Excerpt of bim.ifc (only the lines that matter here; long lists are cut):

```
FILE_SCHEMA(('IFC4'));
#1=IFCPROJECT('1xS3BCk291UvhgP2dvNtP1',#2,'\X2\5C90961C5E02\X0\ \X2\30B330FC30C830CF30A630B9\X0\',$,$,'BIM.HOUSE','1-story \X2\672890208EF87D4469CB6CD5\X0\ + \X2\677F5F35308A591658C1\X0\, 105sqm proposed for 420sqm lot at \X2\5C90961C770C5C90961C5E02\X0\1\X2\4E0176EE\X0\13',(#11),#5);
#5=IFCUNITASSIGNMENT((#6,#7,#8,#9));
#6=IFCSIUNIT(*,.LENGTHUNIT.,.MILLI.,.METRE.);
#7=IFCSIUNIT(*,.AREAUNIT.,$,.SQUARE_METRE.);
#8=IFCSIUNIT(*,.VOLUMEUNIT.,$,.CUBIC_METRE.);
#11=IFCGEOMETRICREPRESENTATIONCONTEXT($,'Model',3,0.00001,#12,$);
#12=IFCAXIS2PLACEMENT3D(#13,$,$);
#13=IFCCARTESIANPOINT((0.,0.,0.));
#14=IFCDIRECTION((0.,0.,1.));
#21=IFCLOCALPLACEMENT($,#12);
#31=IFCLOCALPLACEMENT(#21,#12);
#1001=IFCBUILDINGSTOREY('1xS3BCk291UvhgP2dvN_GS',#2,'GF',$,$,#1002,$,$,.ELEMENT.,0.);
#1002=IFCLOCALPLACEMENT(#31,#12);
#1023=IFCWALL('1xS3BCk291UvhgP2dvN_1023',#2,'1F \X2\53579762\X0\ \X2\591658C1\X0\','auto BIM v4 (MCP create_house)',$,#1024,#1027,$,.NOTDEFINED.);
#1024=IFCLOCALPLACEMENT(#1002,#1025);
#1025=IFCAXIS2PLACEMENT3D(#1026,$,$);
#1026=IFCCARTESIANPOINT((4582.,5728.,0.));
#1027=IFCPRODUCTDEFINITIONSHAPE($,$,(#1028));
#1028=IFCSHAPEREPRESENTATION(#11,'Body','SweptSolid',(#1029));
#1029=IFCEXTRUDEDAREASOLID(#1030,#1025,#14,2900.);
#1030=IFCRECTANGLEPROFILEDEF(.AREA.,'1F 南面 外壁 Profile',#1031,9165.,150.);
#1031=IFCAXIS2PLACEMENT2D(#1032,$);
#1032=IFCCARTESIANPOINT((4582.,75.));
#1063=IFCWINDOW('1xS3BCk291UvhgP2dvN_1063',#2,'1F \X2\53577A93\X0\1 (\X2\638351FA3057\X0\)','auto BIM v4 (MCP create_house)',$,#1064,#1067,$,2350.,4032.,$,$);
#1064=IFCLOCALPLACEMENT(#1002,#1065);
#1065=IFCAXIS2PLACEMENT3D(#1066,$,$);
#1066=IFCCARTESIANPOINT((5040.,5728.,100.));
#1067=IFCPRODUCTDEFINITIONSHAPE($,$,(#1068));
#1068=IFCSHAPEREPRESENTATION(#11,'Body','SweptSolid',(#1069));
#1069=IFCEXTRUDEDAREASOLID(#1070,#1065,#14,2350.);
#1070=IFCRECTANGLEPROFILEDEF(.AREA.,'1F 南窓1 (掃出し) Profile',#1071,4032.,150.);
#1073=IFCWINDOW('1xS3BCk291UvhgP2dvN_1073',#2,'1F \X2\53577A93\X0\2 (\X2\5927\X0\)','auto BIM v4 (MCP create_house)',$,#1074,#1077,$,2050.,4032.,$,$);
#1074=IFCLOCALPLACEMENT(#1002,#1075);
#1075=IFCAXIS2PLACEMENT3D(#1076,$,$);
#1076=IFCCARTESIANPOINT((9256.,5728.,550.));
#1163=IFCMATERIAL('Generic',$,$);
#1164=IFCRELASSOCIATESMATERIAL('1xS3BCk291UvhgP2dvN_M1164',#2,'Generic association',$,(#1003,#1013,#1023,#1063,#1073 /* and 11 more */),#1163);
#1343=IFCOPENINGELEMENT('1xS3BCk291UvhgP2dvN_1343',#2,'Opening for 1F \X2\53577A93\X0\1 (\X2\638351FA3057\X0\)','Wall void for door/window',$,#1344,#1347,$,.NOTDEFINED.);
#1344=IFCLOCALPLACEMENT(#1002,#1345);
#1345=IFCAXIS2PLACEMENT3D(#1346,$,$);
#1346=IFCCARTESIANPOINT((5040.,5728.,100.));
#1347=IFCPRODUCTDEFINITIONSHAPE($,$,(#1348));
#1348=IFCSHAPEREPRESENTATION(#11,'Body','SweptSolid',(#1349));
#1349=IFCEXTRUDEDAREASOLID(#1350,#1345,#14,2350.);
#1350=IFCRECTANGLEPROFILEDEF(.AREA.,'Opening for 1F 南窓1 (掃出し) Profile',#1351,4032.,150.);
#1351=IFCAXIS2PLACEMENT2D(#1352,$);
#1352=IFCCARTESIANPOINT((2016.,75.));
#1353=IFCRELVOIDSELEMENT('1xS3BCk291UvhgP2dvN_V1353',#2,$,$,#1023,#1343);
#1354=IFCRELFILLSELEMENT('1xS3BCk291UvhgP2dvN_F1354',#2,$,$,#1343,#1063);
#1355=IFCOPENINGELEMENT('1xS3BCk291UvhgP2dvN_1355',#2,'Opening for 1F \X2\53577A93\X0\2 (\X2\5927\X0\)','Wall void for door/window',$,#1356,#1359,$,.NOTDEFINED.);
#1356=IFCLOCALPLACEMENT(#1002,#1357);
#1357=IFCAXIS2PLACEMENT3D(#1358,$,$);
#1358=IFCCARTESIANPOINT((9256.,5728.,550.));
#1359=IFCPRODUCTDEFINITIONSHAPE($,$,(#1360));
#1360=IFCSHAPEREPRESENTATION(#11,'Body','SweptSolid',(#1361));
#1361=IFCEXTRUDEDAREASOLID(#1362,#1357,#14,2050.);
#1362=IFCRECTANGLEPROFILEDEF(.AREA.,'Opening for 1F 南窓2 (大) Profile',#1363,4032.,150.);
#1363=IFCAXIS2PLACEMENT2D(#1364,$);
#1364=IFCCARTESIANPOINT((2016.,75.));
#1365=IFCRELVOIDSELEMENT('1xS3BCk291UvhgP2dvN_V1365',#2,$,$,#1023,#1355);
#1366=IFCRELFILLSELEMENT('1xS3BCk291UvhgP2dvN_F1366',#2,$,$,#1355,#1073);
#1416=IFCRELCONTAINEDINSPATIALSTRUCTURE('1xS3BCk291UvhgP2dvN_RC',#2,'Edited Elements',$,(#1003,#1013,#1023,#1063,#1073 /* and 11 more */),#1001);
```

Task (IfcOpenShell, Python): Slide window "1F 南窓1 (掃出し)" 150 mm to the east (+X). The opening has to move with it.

```python
import ifcopenshell
import ifcopenshell.api.geometry
import ifcopenshell.util.placement
import ifcopenshell.util.unit

model = ifcopenshell.open("bim.ifc")
unit_scale = ifcopenshell.util.unit.calculate_unit_scale(model)

window = model.by_guid("1xS3BCk291UvhgP2dvN_1063")
opening = window.FillsVoids[0].RelatingOpeningElement
wall = opening.VoidsElements[0].RelatingBuildingElement

wall_matrix = ifcopenshell.util.placement.get_local_placement(wall.ObjectPlacement)
shift = wall_matrix[:3, 0] * 0.15 / unit_scale
before = ifcopenshell.util.placement.get_local_placement(window.ObjectPlacement)[:3, 3].copy()

# The window is not placed relative to its opening, so move both.
for product in (opening, window):
    matrix = ifcopenshell.util.placement.get_local_placement(product.ObjectPlacement)
    matrix[:3, 3] += shift
    ifcopenshell.api.geometry.edit_object_placement(model, product=product, matrix=matrix, is_si=False)

after = ifcopenshell.util.placement.get_local_placement(window.ObjectPlacement)[:3, 3]
print("window moved by", (after - before).round(3) + 0.0)

model.write("bim_v2.ifc")
```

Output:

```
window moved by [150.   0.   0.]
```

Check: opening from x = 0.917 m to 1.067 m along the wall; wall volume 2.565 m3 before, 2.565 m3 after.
